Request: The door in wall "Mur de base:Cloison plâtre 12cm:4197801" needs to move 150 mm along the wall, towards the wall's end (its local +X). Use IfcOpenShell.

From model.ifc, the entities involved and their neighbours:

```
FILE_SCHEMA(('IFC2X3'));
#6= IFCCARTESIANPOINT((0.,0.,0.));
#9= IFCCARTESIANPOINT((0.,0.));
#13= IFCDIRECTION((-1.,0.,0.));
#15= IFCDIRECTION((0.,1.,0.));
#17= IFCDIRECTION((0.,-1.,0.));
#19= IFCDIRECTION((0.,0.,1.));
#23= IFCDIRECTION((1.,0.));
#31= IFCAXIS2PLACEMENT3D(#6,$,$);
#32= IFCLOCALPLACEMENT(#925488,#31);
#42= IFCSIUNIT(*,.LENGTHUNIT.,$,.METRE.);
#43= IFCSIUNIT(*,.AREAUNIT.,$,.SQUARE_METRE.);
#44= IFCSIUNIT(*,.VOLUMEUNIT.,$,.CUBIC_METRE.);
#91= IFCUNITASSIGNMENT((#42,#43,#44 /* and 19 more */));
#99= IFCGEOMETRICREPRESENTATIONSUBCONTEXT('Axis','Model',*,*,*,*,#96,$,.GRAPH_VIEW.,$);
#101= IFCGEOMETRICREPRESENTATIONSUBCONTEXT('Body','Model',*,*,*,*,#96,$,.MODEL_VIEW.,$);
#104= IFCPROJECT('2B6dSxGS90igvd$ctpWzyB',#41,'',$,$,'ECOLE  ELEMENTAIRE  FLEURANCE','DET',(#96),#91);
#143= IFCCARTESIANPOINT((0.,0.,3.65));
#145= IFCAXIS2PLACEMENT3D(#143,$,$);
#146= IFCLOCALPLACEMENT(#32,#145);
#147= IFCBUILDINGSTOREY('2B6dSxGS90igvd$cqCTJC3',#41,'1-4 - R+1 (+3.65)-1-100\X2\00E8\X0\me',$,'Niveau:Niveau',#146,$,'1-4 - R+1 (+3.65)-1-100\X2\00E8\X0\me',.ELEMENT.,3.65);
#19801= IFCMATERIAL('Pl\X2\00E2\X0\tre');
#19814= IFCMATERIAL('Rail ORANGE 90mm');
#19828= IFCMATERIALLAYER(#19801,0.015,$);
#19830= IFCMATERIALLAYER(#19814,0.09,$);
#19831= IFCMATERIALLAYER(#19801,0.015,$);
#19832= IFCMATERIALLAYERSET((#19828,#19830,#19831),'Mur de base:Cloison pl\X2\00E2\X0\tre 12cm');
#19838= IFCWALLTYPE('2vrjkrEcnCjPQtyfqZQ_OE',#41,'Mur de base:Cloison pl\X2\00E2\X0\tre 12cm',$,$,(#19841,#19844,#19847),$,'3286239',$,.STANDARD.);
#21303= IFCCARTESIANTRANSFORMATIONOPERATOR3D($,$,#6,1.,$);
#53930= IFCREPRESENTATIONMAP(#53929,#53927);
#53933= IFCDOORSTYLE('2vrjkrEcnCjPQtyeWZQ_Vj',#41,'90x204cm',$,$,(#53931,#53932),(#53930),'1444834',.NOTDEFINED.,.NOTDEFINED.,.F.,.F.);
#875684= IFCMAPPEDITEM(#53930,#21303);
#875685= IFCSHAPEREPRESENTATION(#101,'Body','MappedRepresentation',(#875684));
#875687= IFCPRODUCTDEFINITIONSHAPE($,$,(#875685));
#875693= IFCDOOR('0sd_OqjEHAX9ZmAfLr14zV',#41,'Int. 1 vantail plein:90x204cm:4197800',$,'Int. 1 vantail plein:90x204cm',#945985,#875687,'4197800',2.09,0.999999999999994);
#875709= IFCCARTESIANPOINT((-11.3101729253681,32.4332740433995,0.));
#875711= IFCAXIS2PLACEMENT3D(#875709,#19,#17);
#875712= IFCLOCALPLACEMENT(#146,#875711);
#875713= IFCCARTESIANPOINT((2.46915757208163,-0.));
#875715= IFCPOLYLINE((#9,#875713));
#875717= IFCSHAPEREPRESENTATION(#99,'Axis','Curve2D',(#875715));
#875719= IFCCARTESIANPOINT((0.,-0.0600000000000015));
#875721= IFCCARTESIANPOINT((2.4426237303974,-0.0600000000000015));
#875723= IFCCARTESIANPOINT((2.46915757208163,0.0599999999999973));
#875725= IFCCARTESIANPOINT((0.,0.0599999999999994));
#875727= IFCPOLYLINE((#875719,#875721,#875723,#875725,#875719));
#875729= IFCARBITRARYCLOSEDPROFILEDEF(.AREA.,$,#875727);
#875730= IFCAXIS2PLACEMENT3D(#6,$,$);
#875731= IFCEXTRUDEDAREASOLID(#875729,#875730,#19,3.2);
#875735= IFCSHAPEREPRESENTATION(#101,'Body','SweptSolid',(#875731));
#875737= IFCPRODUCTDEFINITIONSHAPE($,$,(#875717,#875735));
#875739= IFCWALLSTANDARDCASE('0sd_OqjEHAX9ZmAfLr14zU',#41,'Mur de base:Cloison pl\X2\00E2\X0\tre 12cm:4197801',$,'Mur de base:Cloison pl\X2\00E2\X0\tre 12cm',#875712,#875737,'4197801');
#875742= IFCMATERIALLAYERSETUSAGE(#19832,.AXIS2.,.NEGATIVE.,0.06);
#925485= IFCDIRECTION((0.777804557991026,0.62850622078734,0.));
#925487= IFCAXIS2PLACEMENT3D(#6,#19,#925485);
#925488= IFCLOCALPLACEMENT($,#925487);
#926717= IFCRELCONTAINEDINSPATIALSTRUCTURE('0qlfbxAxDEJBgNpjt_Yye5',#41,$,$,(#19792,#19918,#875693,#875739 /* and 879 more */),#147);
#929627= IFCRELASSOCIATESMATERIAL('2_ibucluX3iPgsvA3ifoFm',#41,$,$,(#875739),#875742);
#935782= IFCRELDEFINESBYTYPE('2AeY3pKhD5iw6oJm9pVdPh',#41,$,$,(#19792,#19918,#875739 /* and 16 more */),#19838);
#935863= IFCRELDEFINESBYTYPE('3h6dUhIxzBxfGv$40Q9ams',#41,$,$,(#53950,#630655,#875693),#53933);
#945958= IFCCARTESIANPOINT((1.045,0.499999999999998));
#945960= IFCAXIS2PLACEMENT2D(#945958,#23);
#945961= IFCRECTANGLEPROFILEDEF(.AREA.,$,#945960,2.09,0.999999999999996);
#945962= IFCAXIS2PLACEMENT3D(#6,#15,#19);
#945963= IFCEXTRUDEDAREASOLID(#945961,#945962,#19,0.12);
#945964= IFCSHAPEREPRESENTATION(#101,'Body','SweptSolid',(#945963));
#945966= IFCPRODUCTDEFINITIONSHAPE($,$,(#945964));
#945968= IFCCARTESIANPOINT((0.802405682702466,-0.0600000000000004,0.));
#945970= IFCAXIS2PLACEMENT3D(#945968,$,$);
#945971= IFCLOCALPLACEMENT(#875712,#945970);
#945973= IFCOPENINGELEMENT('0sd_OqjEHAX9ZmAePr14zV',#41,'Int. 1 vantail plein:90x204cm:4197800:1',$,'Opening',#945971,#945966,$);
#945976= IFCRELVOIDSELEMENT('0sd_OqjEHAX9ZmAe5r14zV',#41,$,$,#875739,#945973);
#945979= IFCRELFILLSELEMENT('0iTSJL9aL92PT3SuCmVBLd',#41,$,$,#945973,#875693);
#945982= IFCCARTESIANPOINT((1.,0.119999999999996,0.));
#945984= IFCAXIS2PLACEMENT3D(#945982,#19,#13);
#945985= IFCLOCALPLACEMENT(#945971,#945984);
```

```python
import ifcopenshell
import ifcopenshell.api.geometry
import ifcopenshell.util.placement

model = ifcopenshell.open("model.ifc")

door = model.by_guid("0sd_OqjEHAX9ZmAfLr14zV")
opening = door.FillsVoids[0].RelatingOpeningElement
wall = opening.VoidsElements[0].RelatingBuildingElement

wall_matrix = ifcopenshell.util.placement.get_local_placement(wall.ObjectPlacement)
shift = wall_matrix[:3, 0] * 0.15
before = ifcopenshell.util.placement.get_local_placement(door.ObjectPlacement)[:3, 3].copy()

# The door is placed relative to its opening, so it follows when the opening moves.
matrix = ifcopenshell.util.placement.get_local_placement(opening.ObjectPlacement)
matrix[:3, 3] += shift
ifcopenshell.api.geometry.edit_object_placement(
    model, product=opening, matrix=matrix, is_si=False, should_transform_children=True
)

after = ifcopenshell.util.placement.get_local_placement(door.ObjectPlacement)[:3, 3]
print("door moved by", (after - before).round(3) + 0.0)

model.write("model-out.ifc")
```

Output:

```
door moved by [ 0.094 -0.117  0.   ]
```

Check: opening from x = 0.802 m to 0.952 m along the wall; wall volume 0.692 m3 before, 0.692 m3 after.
